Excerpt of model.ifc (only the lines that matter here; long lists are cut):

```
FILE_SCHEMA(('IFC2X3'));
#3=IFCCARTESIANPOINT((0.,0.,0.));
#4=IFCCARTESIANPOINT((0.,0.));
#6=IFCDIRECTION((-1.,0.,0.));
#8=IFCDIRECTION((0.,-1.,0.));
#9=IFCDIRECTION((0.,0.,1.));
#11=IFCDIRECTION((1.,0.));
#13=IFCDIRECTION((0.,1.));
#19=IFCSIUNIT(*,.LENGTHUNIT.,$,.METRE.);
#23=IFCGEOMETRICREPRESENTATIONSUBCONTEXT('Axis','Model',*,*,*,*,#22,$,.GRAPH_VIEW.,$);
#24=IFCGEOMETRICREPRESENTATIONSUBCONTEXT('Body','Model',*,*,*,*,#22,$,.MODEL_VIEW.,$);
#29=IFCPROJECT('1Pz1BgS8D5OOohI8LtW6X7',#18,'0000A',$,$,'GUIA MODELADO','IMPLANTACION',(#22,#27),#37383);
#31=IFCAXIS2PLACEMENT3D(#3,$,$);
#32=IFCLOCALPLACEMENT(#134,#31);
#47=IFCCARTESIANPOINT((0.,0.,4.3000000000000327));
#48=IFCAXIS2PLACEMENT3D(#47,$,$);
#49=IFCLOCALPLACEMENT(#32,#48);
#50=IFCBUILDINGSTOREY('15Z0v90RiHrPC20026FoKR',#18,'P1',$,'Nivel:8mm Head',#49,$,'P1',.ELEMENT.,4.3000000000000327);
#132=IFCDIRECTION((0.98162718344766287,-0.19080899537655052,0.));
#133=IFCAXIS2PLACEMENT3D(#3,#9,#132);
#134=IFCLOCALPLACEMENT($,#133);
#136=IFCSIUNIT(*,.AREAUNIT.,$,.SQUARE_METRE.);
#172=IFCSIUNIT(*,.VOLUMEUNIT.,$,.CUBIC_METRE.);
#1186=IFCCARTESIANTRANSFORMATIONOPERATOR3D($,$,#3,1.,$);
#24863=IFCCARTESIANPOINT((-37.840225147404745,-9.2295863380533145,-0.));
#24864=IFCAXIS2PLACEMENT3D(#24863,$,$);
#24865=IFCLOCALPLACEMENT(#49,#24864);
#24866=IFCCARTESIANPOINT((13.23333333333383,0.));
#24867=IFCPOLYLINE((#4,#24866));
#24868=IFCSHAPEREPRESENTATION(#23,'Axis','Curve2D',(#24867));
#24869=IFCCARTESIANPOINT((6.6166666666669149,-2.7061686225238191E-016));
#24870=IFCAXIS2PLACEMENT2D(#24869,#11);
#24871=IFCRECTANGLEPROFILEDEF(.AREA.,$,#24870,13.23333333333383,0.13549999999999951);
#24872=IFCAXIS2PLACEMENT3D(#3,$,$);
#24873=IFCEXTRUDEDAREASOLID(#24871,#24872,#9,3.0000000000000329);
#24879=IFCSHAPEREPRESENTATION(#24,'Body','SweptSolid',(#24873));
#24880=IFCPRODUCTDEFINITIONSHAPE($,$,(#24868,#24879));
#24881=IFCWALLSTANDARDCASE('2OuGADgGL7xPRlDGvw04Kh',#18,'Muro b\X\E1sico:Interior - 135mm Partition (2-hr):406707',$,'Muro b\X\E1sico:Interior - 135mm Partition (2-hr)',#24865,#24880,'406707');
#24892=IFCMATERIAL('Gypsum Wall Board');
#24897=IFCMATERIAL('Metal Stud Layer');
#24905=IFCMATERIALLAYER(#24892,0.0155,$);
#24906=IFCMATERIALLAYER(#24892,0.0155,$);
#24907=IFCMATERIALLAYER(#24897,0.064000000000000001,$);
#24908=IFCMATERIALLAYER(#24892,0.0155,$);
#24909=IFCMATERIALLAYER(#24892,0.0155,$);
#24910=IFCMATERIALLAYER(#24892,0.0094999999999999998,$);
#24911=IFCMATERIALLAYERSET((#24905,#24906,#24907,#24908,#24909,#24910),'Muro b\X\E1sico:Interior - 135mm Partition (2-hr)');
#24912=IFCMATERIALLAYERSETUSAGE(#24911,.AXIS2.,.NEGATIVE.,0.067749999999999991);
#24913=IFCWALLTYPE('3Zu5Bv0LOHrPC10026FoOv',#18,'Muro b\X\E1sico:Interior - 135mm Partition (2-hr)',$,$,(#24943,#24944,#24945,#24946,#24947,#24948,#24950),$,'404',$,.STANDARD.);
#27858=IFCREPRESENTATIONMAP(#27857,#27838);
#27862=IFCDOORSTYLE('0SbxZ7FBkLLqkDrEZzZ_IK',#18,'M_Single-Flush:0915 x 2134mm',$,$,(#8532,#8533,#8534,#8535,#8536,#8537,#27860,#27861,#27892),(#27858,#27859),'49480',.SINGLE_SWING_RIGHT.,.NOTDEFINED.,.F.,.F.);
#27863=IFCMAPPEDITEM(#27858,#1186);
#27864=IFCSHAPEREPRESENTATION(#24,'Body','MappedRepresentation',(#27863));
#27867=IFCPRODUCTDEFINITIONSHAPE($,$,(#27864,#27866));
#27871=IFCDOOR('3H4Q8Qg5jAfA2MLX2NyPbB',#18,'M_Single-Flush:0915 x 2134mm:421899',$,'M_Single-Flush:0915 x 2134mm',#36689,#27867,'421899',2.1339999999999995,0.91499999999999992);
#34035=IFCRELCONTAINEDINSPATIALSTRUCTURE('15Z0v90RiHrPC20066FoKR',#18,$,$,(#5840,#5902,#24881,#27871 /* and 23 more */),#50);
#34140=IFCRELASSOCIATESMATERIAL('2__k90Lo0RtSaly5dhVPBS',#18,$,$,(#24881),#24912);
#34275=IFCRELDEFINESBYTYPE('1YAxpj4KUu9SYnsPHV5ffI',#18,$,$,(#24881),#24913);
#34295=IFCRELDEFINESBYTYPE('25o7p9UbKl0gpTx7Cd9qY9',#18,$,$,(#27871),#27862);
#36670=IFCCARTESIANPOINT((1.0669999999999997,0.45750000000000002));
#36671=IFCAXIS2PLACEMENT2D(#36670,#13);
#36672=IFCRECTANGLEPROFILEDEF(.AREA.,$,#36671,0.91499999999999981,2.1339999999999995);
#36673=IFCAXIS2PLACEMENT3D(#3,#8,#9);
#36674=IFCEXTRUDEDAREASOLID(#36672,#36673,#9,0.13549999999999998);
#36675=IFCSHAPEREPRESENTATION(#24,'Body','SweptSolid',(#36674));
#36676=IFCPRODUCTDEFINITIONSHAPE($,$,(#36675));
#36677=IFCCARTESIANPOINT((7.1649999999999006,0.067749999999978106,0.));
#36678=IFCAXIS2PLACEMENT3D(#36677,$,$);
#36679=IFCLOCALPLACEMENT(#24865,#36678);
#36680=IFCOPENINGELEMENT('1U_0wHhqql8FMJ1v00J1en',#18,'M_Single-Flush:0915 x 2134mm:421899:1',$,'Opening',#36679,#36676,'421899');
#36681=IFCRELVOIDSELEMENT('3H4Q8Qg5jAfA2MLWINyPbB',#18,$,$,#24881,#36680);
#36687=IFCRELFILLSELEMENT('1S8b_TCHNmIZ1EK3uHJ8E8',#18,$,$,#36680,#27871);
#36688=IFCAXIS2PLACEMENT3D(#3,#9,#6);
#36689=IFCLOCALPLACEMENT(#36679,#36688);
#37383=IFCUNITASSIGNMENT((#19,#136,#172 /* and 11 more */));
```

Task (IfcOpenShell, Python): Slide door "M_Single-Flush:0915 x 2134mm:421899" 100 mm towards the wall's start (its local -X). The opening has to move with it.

```python
import ifcopenshell
import ifcopenshell.api.geometry
import ifcopenshell.util.placement
import ifcopenshell.util.unit

model = ifcopenshell.open("model.ifc")
unit_scale = ifcopenshell.util.unit.calculate_unit_scale(model)

door = model.by_guid("3H4Q8Qg5jAfA2MLX2NyPbB")
opening = door.FillsVoids[0].RelatingOpeningElement
wall = opening.VoidsElements[0].RelatingBuildingElement

wall_matrix = ifcopenshell.util.placement.get_local_placement(wall.ObjectPlacement)
shift = wall_matrix[:3, 0] * -0.1 / unit_scale
before = ifcopenshell.util.placement.get_local_placement(door.ObjectPlacement)[:3, 3].copy()

# The door is placed relative to its opening, so it follows when the opening moves.
matrix = ifcopenshell.util.placement.get_local_placement(opening.ObjectPlacement)
matrix[:3, 3] += shift
ifcopenshell.api.geometry.edit_object_placement(
    model, product=opening, matrix=matrix, is_si=False, should_transform_children=True
)

after = ifcopenshell.util.placement.get_local_placement(door.ObjectPlacement)[:3, 3]
print("door moved by", (after - before).round(3) + 0.0)

model.write("model_v2.ifc")
```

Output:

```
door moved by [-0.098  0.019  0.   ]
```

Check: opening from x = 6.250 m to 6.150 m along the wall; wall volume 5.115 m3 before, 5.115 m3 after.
